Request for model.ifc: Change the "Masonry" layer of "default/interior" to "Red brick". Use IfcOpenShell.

First a look at what the model holds.

```python
import ifcopenshell
import ifcopenshell.util.element

model = ifcopenshell.open("model.ifc")
print(model.schema)
for layer_set in model.by_type("IfcMaterialLayerSet"):
    if layer_set.LayerSetName == "default/interior":
        for layer in layer_set.MaterialLayers:
            print(layer.id(), layer.Material and layer.Material.Name, layer.LayerThickness, sep=" | ")
        print(len(ifcopenshell.util.element.get_elements_by_material(model, layer_set)), "elements and types use it")
print(sorted(m.Name for m in model.by_type("IfcMaterial") if m.Name)[:60])
```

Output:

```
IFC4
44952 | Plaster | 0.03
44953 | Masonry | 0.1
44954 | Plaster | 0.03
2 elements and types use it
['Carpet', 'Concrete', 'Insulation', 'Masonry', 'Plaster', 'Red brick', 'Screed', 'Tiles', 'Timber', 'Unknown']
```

```python
import ifcopenshell
import ifcopenshell.api.material

model = ifcopenshell.open("model.ifc")

layer_set = next(s for s in model.by_type("IfcMaterialLayerSet") if s.LayerSetName == "default/interior")
layer = next(l for l in layer_set.MaterialLayers if l.Material and l.Material.Name == "Masonry")
material = next(m for m in model.by_type("IfcMaterial") if m.Name == "Red brick")

# Point this one layer at the other material; renaming the old one would change it everywhere.
ifcopenshell.api.material.edit_layer(model, layer=layer, attributes={"Name": material.Name}, material=material)

print([l.Material.Name if l.Material else None for l in layer_set.MaterialLayers])

model.write("model-out.ifc")
```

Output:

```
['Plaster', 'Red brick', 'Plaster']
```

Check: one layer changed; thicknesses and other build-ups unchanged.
